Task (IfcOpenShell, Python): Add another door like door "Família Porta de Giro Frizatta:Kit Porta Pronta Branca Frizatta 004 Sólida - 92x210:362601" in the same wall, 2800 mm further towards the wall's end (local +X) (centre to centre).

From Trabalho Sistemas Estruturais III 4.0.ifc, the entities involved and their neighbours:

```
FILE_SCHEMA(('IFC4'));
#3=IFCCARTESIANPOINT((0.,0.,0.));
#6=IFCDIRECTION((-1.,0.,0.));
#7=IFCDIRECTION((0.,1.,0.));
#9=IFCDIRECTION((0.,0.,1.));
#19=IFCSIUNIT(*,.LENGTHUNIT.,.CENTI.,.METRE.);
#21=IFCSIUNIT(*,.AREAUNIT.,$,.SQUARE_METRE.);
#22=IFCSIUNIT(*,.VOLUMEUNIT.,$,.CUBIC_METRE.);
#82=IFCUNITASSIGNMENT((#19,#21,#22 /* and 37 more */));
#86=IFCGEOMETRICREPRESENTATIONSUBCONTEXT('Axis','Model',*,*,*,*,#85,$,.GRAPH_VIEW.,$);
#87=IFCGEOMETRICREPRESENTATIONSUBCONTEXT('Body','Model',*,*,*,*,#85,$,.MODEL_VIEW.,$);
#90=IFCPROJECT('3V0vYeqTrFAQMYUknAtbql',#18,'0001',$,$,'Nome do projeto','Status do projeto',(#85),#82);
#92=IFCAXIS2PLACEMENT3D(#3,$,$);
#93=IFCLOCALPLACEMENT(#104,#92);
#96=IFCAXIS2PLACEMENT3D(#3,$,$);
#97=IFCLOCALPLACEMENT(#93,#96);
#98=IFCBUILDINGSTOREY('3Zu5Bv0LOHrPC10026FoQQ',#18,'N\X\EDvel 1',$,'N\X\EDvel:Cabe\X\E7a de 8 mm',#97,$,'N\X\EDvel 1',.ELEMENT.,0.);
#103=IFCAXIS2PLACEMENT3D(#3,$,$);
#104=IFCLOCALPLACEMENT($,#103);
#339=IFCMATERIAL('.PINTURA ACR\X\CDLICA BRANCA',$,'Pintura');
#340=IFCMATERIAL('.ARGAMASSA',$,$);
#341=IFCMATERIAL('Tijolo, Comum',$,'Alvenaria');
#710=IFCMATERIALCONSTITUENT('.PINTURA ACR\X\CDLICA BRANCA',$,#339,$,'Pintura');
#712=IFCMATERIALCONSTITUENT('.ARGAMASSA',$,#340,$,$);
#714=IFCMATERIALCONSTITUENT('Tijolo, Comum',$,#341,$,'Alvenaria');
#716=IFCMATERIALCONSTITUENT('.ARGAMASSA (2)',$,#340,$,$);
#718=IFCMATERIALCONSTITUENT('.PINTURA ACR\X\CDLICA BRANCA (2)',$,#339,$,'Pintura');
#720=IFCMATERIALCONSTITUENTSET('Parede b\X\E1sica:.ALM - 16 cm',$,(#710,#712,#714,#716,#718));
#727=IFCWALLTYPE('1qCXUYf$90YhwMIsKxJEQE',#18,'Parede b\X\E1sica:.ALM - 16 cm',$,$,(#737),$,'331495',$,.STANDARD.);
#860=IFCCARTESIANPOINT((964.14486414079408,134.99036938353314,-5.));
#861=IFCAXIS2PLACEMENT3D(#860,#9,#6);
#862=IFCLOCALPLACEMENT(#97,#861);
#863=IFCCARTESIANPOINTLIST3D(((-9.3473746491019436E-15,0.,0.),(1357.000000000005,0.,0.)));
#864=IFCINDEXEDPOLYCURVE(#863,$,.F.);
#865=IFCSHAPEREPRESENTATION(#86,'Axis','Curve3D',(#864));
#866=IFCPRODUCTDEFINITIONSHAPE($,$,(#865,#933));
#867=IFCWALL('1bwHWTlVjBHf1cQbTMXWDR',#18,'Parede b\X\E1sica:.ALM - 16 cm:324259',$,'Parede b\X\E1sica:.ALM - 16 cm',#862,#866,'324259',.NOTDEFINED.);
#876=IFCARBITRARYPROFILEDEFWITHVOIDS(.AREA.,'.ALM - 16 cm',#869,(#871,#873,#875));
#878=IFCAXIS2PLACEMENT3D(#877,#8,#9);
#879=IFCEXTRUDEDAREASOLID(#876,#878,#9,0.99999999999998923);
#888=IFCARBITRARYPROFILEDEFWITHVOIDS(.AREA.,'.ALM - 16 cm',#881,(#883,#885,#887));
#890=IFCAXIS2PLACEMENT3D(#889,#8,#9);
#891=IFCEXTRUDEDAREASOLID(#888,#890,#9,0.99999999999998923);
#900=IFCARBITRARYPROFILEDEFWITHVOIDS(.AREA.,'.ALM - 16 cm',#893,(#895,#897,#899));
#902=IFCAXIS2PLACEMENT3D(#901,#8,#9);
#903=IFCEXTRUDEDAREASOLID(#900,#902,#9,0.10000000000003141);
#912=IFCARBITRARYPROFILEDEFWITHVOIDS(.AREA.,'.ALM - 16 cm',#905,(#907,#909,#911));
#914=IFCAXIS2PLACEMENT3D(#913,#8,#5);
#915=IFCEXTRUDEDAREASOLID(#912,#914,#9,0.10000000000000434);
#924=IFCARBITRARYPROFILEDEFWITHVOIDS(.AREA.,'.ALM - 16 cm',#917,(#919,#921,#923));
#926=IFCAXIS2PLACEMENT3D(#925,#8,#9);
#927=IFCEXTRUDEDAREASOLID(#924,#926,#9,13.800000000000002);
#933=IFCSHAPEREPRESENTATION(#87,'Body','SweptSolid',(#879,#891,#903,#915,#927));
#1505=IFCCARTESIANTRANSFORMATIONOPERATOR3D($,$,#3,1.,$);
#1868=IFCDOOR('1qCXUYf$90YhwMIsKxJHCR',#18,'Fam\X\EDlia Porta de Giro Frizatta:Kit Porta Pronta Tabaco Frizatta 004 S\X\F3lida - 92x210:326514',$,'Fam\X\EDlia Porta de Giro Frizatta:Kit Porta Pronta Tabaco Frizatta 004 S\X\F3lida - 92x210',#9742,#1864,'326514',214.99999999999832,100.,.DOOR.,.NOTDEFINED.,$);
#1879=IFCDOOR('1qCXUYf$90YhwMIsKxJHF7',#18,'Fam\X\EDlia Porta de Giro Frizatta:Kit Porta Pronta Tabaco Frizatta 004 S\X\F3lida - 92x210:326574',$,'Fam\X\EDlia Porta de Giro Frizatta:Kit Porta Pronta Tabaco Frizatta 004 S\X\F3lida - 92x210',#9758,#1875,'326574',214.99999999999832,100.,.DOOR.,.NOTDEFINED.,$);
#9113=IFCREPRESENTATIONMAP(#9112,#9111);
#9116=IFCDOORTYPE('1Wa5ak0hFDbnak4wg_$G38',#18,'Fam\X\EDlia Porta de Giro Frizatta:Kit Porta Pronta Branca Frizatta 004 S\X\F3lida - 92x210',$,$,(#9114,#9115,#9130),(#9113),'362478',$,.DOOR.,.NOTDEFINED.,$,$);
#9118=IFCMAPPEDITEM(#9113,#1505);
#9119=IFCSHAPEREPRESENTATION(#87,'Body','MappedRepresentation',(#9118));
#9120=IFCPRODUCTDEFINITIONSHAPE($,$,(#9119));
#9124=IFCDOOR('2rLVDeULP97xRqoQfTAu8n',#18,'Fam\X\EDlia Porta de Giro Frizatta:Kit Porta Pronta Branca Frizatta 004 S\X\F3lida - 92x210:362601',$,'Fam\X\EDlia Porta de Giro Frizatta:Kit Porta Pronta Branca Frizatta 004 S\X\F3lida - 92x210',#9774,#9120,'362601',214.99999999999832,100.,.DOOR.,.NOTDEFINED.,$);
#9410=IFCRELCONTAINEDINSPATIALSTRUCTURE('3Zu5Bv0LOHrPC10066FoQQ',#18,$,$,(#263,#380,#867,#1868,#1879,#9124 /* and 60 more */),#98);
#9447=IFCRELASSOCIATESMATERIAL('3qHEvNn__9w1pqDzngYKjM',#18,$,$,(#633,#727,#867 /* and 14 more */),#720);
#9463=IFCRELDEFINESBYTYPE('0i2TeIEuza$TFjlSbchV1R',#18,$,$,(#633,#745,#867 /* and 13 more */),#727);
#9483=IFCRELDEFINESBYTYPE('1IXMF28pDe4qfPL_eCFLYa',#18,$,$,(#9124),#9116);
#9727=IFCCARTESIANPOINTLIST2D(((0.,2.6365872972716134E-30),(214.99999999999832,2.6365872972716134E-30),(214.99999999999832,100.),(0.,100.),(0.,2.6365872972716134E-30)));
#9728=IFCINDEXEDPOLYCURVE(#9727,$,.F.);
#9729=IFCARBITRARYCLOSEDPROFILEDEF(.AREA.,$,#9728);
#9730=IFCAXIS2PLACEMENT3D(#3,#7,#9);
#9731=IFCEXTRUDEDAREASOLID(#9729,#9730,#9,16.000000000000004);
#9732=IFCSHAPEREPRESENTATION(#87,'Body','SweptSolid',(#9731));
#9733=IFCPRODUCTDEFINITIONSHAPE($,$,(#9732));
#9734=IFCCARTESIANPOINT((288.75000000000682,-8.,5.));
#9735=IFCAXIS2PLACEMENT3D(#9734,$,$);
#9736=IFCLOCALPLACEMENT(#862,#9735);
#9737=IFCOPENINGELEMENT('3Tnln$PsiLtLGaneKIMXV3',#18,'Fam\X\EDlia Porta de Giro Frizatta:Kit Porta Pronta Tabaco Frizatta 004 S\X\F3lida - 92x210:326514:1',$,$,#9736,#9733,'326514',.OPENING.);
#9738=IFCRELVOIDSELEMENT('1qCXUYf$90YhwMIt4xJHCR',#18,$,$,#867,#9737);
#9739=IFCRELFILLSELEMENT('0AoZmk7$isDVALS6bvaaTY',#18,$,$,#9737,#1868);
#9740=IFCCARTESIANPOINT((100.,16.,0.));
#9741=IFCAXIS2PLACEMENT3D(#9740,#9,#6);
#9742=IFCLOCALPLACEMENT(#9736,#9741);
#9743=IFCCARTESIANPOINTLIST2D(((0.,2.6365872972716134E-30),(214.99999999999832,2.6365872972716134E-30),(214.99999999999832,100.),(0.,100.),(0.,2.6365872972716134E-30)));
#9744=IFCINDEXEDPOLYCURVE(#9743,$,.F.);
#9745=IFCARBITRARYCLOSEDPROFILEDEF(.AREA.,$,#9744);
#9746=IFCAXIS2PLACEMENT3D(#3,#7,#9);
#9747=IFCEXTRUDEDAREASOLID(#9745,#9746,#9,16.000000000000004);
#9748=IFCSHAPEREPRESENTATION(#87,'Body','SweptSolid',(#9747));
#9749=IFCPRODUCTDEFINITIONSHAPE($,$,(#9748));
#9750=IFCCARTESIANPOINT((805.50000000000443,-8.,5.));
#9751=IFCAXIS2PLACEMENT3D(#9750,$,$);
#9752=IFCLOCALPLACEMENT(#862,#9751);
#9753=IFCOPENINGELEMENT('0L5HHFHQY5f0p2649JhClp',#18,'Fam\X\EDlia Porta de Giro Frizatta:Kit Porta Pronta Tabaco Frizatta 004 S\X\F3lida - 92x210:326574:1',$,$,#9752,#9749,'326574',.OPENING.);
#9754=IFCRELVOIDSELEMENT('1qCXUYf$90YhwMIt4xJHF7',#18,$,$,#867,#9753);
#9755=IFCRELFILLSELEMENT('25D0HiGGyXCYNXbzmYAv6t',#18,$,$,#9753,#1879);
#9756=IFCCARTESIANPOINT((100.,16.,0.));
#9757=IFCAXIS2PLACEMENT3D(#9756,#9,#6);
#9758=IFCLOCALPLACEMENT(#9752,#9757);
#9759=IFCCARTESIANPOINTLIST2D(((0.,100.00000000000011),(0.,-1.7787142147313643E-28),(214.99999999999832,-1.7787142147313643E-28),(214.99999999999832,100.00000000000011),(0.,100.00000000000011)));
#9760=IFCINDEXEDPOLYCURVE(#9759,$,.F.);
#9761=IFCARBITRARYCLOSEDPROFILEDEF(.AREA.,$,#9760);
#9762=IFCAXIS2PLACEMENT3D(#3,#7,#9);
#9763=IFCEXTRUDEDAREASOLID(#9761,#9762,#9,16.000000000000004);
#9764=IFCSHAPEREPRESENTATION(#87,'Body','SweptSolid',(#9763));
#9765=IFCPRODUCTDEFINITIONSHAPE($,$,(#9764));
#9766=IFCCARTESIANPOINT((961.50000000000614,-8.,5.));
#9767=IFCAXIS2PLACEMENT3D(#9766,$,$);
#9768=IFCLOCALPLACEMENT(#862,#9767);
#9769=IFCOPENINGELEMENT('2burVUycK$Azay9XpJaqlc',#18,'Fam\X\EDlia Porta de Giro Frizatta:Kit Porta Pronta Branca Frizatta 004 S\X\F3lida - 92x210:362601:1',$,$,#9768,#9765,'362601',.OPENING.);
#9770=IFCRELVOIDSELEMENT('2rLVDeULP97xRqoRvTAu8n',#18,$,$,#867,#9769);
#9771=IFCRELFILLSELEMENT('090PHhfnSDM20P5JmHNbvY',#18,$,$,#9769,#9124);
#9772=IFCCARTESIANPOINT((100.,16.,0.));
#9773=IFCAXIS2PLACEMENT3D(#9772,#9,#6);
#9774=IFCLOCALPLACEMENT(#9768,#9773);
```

```python
import ifcopenshell
import ifcopenshell.api.feature
import ifcopenshell.api.geometry
import ifcopenshell.api.root
import ifcopenshell.geom
import ifcopenshell.util.element
import ifcopenshell.util.placement
import ifcopenshell.util.shape
import ifcopenshell.util.unit

model = ifcopenshell.open("Trabalho Sistemas Estruturais III 4.0.ifc")
unit_scale = ifcopenshell.util.unit.calculate_unit_scale(model)
settings = ifcopenshell.geom.settings()


def volume(element):
    """Net volume in cubic metres, openings subtracted."""
    shape = ifcopenshell.geom.create_shape(settings, element)
    return ifcopenshell.util.shape.get_volume(shape.geometry)


def reuse_history(source, copy):
    """copy_class also copies each property set's owner history, people and application; keep the originals."""
    for rel in copy.IsDefinedBy:
        if rel.is_a("IfcRelDefinesByProperties") and (history := rel.RelatingPropertyDefinition.OwnerHistory):
            rel.RelatingPropertyDefinition.OwnerHistory = source.OwnerHistory
            ifcopenshell.util.element.remove_deep2(model, history)


door = model.by_guid("2rLVDeULP97xRqoQfTAu8n")
opening = door.FillsVoids[0].RelatingOpeningElement
wall = opening.VoidsElements[0].RelatingBuildingElement
before = volume(wall)
shift = ifcopenshell.util.placement.get_local_placement(wall.ObjectPlacement)[:3, 0] * 2.8 / unit_scale

# copy_class copies the void relationship, type, container and properties, but no geometry.
new_opening = ifcopenshell.api.root.copy_class(model, product=opening)
new_opening.Representation = ifcopenshell.util.element.copy_deep(
    model, opening.Representation, exclude=["IfcGeometricRepresentationContext", "IfcRepresentationMap"]
)
new_opening.Name = "Família Porta de Giro Frizatta:Kit Porta Pronta Branca Frizatta 004 Sólida - 92x210"
new_opening.Tag = None
new_door = ifcopenshell.api.root.copy_class(model, product=door)
new_door.Representation = ifcopenshell.util.element.copy_deep(
    model, door.Representation, exclude=["IfcGeometricRepresentationContext", "IfcRepresentationMap"]
)
new_door.Name = "Família Porta de Giro Frizatta:Kit Porta Pronta Branca Frizatta 004 Sólida - 92x210"
new_door.Tag = None
reuse_history(door, new_door)
ifcopenshell.api.feature.add_filling(model, opening=new_opening, element=new_door)

for old, new in ((opening, new_opening), (door, new_door)):
    matrix = ifcopenshell.util.placement.get_local_placement(old.ObjectPlacement)
    matrix[:3, 3] += shift
    ifcopenshell.api.geometry.edit_object_placement(model, product=new, matrix=matrix, is_si=False)

after = volume(wall)

print(f"wall volume {before:.3f} -> {after:.3f} m3")

model.write("Trabalho Sistemas Estruturais III 4.0_edited.ifc")
```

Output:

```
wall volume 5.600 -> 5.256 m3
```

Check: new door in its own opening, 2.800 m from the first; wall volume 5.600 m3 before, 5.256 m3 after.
